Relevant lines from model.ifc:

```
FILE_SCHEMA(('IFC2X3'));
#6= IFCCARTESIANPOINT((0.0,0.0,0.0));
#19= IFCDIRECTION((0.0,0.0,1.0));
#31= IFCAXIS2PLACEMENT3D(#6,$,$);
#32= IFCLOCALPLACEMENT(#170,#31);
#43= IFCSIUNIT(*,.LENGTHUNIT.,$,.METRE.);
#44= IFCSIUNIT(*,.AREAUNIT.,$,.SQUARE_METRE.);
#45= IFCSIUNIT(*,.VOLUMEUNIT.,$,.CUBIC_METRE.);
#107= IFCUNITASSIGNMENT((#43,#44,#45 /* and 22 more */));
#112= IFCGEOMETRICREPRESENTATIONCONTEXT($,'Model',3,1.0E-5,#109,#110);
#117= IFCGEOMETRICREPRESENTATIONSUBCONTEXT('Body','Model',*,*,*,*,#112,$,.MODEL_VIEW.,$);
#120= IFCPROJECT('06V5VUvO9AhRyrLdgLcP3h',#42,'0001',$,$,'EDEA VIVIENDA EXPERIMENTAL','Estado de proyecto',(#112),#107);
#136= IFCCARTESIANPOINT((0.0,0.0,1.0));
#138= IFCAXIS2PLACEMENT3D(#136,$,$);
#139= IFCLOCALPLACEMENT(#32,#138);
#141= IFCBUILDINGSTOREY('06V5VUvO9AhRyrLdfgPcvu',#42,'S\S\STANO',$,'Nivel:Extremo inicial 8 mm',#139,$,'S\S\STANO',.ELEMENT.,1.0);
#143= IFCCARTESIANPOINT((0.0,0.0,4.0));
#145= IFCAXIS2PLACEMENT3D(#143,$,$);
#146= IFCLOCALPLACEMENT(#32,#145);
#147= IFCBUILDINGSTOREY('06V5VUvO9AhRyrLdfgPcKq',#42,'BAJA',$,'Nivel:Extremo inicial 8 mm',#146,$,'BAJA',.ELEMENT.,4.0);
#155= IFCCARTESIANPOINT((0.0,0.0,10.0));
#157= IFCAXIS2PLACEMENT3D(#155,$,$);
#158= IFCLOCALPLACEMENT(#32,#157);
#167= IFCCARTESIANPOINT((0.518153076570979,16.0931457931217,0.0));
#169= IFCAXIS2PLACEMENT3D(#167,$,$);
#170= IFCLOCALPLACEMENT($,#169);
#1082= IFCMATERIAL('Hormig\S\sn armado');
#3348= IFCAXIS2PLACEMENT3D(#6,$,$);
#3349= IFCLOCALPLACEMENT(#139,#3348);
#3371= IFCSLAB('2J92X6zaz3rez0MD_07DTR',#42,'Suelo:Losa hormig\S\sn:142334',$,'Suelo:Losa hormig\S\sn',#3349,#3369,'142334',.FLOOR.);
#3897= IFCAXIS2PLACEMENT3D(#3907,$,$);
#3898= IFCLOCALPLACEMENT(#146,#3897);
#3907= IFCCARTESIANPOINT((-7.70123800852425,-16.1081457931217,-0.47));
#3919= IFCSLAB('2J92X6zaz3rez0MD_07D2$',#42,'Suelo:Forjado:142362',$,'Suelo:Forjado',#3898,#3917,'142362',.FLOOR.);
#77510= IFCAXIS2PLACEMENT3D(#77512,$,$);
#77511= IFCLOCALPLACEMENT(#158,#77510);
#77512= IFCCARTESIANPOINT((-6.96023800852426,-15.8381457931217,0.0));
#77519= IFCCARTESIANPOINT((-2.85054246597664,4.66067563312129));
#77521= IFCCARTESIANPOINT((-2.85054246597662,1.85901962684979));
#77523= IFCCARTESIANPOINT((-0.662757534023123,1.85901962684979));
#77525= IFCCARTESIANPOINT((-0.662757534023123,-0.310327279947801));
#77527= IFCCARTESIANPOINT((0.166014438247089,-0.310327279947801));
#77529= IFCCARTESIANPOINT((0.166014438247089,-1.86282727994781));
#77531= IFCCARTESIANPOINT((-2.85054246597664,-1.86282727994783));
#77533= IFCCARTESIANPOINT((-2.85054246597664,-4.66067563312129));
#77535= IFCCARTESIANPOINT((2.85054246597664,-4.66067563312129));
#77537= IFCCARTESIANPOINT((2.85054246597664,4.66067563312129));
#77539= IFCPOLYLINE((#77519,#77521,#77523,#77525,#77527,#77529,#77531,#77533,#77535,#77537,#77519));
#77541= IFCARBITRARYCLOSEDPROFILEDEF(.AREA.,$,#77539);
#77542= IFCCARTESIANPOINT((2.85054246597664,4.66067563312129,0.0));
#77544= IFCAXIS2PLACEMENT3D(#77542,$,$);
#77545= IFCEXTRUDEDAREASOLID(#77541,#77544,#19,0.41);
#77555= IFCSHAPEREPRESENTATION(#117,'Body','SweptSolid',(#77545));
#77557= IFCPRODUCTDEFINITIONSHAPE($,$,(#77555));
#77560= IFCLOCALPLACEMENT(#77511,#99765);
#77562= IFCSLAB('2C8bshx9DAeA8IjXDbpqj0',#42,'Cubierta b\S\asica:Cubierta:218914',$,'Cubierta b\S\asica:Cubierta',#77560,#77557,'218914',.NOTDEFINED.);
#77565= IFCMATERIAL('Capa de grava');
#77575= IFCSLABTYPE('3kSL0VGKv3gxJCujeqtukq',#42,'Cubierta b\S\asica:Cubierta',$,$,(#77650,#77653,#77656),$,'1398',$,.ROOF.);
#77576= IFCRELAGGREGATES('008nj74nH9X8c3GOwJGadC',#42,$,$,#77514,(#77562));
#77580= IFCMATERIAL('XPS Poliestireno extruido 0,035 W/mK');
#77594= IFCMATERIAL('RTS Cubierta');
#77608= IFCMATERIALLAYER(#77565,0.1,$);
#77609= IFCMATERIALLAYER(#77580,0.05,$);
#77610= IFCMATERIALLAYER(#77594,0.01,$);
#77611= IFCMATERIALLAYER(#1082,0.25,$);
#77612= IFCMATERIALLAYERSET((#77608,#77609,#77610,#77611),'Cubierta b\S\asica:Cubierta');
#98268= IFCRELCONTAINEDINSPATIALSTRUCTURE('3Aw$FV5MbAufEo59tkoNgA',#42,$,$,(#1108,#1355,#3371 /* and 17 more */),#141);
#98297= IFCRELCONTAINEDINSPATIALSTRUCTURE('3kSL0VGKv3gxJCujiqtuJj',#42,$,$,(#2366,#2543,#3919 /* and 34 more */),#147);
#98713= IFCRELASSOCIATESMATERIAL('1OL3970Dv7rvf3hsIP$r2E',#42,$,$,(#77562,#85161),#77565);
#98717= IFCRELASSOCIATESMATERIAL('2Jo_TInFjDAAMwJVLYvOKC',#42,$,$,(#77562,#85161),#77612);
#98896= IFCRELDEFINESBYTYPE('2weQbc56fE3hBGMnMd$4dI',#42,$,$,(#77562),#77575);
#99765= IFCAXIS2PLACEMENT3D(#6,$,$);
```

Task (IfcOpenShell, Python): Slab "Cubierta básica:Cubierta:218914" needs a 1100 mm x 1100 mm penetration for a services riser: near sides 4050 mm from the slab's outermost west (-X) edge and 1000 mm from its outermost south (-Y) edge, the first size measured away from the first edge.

```python
import numpy as np
import ifcopenshell
import ifcopenshell.api.feature
import ifcopenshell.api.geometry
import ifcopenshell.api.root
import ifcopenshell.geom
import ifcopenshell.util.placement
import ifcopenshell.util.representation
import ifcopenshell.util.shape
import ifcopenshell.util.unit

model = ifcopenshell.open("model.ifc")
unit_scale = ifcopenshell.util.unit.calculate_unit_scale(model)
settings = ifcopenshell.geom.settings()


def volume(element):
    """Net volume in cubic metres, openings subtracted."""
    shape = ifcopenshell.geom.create_shape(settings, element)
    return ifcopenshell.util.shape.get_volume(shape.geometry)


slab = model.by_guid("2C8bshx9DAeA8IjXDbpqj0")
before = volume(slab)

# Extent in the slab's own axes, in metres. The edges named are its -X and -Y sides.
slab_shape = ifcopenshell.geom.create_shape(settings, slab)
vertices = ifcopenshell.util.shape.get_vertices(slab_shape.geometry)
x_min, y_min, bottom = vertices.min(axis=0)
top = vertices[:, 2].max()

opening = ifcopenshell.api.root.create_entity(model, ifc_class="IfcOpeningElement", name="Services riser opening")
context = ifcopenshell.util.representation.get_context(model, "Model", "Body", "MODEL_VIEW")
width, depth = 1.1, 1.1
outline = [(0.0, 0.0), (width, 0.0), (width, depth), (0.0, depth), (0.0, 0.0)]
# Overshoot both faces by 50 mm so the cut is clean.
shape = ifcopenshell.api.geometry.add_slab_representation(
    model, context=context, depth=top - bottom + 0.1, polyline=outline
)
ifcopenshell.api.geometry.assign_representation(model, product=opening, representation=shape)

matrix = ifcopenshell.util.placement.get_local_placement(slab.ObjectPlacement)
matrix[:, 3] = matrix @ np.append(np.array([x_min + 4.05, y_min + 1, bottom - 0.05]) / unit_scale, 1.0)
ifcopenshell.api.geometry.edit_object_placement(model, product=opening, matrix=matrix, is_si=False)
ifcopenshell.api.feature.add_feature(model, feature=opening, element=slab)

after = volume(slab)

print(f"slab volume {before:.3f} -> {after:.3f} m3")

model.write("model_updated.ifc")
```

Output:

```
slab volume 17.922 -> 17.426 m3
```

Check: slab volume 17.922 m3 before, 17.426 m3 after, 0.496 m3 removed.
